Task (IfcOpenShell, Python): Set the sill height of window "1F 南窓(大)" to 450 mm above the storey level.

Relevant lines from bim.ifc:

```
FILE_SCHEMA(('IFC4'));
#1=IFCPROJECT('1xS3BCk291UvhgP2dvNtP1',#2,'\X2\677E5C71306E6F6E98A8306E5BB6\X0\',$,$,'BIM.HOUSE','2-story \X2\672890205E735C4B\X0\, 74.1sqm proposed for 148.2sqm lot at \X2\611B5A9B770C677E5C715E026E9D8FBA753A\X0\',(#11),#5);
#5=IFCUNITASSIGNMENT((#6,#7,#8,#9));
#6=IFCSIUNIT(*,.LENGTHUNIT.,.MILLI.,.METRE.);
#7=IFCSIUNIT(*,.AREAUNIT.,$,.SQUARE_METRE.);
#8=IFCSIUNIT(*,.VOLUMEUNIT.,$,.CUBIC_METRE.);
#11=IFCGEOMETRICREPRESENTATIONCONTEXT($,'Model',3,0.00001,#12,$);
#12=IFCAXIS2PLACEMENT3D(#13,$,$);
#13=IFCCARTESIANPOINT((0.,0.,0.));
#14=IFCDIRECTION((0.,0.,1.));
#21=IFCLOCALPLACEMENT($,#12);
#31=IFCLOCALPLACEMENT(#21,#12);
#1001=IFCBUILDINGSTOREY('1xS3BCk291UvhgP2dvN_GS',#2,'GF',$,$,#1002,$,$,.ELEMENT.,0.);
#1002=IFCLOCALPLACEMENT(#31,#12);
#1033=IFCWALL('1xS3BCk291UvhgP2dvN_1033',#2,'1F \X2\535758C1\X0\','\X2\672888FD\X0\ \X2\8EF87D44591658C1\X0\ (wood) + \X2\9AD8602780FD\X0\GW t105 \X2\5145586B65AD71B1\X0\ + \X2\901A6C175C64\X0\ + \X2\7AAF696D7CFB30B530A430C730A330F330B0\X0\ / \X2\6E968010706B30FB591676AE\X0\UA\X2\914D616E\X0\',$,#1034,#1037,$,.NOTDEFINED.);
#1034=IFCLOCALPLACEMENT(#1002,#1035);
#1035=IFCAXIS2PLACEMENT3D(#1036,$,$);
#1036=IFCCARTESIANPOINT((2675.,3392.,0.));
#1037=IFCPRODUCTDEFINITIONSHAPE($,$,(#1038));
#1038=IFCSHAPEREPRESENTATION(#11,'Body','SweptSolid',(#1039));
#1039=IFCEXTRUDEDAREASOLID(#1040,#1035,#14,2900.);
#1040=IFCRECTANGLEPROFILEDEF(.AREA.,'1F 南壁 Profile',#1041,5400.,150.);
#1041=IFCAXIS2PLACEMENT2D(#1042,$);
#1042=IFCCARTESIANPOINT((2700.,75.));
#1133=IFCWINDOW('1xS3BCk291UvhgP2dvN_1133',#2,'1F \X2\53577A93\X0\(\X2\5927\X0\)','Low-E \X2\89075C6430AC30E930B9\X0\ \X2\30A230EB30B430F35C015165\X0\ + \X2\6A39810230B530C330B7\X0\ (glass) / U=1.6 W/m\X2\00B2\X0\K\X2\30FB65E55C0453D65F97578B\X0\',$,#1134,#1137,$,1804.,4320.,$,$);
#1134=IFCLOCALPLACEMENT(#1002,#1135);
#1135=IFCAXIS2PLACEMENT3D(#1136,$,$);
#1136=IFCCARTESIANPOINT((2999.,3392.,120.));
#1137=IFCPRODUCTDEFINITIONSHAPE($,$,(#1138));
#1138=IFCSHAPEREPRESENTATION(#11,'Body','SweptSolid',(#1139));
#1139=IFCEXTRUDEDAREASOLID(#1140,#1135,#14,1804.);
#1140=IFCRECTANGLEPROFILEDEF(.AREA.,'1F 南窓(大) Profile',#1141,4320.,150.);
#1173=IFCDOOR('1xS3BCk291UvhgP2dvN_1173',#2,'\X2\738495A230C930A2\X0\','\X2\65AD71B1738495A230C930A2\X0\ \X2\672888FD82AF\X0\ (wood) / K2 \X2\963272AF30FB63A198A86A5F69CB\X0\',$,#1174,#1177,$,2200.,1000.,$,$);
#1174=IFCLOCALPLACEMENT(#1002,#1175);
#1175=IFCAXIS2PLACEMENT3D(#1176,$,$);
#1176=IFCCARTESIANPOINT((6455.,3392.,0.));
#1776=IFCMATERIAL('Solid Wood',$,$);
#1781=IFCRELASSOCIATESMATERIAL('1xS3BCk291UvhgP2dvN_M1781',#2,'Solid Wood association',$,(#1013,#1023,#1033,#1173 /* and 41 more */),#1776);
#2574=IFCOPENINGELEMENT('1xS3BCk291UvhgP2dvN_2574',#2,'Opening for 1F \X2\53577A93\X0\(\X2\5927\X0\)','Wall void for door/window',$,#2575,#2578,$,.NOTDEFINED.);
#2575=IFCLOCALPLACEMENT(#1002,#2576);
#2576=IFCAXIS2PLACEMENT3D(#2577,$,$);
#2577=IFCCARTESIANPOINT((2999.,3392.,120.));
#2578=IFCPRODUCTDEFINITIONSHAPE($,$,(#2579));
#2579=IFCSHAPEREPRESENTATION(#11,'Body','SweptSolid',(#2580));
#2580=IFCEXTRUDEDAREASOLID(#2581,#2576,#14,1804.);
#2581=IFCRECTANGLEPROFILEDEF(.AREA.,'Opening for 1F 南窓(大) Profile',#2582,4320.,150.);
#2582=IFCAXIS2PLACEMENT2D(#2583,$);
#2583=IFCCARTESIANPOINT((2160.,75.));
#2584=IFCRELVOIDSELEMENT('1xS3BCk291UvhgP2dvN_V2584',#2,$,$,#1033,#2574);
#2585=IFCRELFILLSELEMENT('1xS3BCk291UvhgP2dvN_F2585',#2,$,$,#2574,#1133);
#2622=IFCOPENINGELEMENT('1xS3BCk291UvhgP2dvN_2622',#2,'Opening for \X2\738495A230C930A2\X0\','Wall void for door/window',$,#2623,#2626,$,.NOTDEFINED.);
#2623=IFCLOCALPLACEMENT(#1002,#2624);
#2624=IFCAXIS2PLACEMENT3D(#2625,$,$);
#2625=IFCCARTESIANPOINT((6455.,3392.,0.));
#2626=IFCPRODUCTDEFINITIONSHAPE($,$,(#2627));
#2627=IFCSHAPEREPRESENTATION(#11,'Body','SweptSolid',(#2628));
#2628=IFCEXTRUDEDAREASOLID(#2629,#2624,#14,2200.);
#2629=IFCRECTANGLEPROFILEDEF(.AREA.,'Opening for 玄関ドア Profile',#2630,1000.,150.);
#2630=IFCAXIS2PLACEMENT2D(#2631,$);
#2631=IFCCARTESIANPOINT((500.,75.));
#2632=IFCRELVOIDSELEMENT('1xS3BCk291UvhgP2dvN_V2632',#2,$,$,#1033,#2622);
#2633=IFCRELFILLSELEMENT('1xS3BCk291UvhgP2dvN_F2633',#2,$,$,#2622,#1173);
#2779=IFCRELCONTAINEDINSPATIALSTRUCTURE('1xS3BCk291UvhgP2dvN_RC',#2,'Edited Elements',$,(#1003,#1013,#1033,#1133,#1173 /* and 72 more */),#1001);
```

```python
import numpy as np
import ifcopenshell
import ifcopenshell.api.geometry
import ifcopenshell.geom
import ifcopenshell.util.element
import ifcopenshell.util.placement
import ifcopenshell.util.shape
import ifcopenshell.util.unit

model = ifcopenshell.open("bim.ifc")
unit_scale = ifcopenshell.util.unit.calculate_unit_scale(model)

window = model.by_guid("1xS3BCk291UvhgP2dvN_1133")
opening = window.FillsVoids[0].RelatingOpeningElement
storey = ifcopenshell.util.element.get_container(window, ifc_class="IfcBuildingStorey")
level = ifcopenshell.util.placement.get_local_placement(storey.ObjectPlacement)[2, 3]

# The opening's origin need not be at the sill, so measure its lowest point.
shape = ifcopenshell.geom.create_shape(ifcopenshell.geom.settings(), opening)
bottom = ifcopenshell.util.shape.get_shape_bottom_elevation(shape, shape.geometry) / unit_scale
dz = level + 450.0 - bottom

shift = np.array([0.0, 0.0, dz])
# The window is not placed relative to its opening, so move both.
for product in (opening, window):
    matrix = ifcopenshell.util.placement.get_local_placement(product.ObjectPlacement)
    matrix[:3, 3] += shift
    ifcopenshell.api.geometry.edit_object_placement(model, product=product, matrix=matrix, is_si=False)

print(f"moved by {dz * unit_scale:+.3f} m")

model.write("bim_v2.ifc")
```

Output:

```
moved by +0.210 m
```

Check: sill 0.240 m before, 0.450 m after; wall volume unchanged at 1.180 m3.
